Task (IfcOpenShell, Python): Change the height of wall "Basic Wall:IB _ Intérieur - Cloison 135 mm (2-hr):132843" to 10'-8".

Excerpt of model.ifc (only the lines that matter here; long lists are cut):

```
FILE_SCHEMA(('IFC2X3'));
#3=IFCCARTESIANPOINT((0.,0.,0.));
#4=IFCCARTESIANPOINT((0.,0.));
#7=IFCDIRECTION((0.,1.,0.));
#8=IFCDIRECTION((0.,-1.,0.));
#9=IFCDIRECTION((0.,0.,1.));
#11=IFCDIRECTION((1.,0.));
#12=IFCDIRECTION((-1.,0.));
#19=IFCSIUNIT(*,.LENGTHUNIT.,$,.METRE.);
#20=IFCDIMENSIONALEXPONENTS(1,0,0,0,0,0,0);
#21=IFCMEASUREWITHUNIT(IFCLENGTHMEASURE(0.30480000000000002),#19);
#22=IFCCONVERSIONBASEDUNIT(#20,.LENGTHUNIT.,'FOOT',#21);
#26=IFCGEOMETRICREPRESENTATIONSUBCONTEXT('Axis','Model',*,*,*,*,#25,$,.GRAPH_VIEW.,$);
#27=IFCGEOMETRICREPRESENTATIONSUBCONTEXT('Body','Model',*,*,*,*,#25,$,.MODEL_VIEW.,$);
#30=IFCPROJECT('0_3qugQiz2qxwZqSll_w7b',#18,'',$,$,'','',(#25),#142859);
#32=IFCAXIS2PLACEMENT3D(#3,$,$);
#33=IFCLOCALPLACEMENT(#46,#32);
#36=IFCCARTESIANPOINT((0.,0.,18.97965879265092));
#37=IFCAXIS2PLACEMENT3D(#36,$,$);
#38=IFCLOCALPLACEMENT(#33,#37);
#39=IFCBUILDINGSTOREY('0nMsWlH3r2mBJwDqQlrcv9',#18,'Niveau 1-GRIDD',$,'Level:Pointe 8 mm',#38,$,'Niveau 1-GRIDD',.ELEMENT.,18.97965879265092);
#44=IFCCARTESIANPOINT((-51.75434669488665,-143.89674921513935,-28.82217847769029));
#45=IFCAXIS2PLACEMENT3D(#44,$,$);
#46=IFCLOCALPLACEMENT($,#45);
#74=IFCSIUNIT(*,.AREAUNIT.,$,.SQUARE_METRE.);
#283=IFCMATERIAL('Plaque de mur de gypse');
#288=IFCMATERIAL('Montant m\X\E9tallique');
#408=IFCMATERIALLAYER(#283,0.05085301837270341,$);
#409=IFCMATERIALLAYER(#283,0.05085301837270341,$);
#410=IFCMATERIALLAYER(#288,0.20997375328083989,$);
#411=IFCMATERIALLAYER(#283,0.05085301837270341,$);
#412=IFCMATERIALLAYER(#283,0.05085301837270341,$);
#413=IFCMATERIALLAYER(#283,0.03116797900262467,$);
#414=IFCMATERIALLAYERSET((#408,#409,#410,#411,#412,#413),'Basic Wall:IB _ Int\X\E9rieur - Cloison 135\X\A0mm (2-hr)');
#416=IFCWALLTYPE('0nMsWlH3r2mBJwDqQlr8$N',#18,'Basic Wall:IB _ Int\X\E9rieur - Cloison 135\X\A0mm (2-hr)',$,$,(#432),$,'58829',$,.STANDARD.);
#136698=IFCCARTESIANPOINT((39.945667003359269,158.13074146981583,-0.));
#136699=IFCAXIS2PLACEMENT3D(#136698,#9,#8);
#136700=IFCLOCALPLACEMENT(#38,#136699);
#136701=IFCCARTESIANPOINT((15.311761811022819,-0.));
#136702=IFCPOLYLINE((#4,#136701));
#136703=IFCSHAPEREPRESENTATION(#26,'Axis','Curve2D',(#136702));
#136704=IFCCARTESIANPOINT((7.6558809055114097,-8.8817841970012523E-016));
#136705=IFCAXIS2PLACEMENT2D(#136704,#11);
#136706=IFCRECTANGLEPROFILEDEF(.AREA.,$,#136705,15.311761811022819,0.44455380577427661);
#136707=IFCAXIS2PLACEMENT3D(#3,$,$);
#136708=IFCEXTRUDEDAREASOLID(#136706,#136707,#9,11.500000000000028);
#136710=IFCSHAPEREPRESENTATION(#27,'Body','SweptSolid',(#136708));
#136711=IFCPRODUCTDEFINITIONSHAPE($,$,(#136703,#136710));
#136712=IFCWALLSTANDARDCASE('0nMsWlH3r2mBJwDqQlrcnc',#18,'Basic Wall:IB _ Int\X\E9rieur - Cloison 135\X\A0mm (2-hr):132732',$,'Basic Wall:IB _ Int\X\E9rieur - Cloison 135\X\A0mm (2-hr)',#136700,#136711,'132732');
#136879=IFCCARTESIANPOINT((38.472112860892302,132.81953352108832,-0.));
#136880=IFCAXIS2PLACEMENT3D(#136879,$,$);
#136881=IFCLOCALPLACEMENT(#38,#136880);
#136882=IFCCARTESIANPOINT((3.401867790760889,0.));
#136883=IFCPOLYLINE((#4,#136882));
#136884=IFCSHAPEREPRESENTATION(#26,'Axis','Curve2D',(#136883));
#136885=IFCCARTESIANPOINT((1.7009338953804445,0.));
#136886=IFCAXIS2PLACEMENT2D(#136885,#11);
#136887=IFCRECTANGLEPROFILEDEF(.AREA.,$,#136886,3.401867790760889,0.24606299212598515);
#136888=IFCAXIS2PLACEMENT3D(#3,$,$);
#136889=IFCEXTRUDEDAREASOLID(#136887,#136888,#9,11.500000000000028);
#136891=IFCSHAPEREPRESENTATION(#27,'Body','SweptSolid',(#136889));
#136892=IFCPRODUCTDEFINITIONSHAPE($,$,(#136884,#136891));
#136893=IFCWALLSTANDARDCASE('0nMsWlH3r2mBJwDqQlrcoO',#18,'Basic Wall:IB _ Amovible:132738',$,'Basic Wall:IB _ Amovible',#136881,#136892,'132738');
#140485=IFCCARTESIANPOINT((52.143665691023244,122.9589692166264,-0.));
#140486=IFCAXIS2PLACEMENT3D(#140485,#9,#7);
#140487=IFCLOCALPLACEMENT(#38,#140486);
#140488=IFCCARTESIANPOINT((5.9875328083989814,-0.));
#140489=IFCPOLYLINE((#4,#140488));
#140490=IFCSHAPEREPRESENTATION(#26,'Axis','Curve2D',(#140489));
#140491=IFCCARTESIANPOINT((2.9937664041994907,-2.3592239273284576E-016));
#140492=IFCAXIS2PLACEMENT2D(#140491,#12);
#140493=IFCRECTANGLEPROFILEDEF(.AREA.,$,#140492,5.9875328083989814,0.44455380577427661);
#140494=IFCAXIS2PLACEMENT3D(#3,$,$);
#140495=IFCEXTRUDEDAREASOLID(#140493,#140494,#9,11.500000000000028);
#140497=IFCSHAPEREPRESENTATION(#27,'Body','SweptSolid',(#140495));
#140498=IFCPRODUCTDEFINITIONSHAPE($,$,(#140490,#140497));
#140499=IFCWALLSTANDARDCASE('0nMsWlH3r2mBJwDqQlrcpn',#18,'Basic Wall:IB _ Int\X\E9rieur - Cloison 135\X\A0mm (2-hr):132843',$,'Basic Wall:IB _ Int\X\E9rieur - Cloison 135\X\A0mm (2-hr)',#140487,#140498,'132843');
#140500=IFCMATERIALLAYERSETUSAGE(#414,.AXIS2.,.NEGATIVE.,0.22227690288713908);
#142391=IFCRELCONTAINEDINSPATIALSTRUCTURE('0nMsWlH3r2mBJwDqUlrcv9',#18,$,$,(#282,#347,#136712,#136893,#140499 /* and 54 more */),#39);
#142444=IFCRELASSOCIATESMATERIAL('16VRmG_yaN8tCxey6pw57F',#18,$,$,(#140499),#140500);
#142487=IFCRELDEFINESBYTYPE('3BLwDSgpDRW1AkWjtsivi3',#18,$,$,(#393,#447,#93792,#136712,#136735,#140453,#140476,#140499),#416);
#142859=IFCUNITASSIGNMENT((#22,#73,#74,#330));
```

```python
import ifcopenshell
import ifcopenshell.geom
import ifcopenshell.util.representation
import ifcopenshell.util.shape
import ifcopenshell.util.unit

model = ifcopenshell.open("model.ifc")
unit_scale = ifcopenshell.util.unit.calculate_unit_scale(model)
settings = ifcopenshell.geom.settings()


def volume(element):
    """Net volume in cubic metres, openings subtracted."""
    shape = ifcopenshell.geom.create_shape(settings, element)
    return ifcopenshell.util.shape.get_volume(shape.geometry)


wall = model.by_guid("0nMsWlH3r2mBJwDqQlrcpn")
before = volume(wall)

body = ifcopenshell.util.representation.get_representation(wall, "Model", "Body")
solid = body.Items[0]
old_height = solid.Depth
solid.Depth = 128 * 0.0254 / unit_scale
after = volume(wall)

print(f"height {old_height:g} -> {solid.Depth:g}, volume {before:.3f} -> {after:.3f} m3")

model.write("model_rev.ifc")
```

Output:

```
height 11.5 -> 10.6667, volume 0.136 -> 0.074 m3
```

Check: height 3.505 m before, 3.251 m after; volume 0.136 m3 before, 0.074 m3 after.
